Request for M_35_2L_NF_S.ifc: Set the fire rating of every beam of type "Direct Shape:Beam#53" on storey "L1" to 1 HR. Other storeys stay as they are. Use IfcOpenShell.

First a look at what the model holds.

```python
import ifcopenshell
import ifcopenshell.util.element

model = ifcopenshell.open("M_35_2L_NF_S.ifc")
print(model.schema)
storey = next(s for s in model.by_type("IfcBuildingStorey") if s.Name == "L1")
beams = [e for e in ifcopenshell.util.element.get_decomposition(storey) if e.is_a("IfcBeam")]
seen = {}
for e in beams:
    element_type = ifcopenshell.util.element.get_type(e)
    key = (element_type.Name if element_type != e and element_type else None, ifcopenshell.util.element.get_pset(e, "Pset_BeamCommon", "FireRating"))
    seen[key] = seen.get(key, 0) + 1
for (name, value), count in sorted(seen.items(), key=str):
    print(count, "x", name, "|", value)
```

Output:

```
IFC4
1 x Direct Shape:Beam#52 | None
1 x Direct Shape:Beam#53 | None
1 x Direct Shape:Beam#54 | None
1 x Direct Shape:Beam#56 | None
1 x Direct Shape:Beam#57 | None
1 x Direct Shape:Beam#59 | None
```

```python
import ifcopenshell
import ifcopenshell.api.pset
import ifcopenshell.util.element

model = ifcopenshell.open("M_35_2L_NF_S.ifc")

storey = next(s for s in model.by_type("IfcBuildingStorey") if s.Name == "L1")
beams = [e for e in ifcopenshell.util.element.get_decomposition(storey) if e.is_a("IfcBeam")]

count = 0
for e in beams:
    element_type = ifcopenshell.util.element.get_type(e)
    if element_type in (None, e) or element_type.Name != "Direct Shape:Beam#53":
        continue
    # add_pset returns the element's existing set when there is one.
    pset = ifcopenshell.api.pset.add_pset(model, product=e, name="Pset_BeamCommon")
    ifcopenshell.api.pset.edit_pset(model, pset=pset, properties={"FireRating": "1 HR"})
    count += 1

print(count, "beams updated")

model.write("M_35_2L_NF_S_updated.ifc")
```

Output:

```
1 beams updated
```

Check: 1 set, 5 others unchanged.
